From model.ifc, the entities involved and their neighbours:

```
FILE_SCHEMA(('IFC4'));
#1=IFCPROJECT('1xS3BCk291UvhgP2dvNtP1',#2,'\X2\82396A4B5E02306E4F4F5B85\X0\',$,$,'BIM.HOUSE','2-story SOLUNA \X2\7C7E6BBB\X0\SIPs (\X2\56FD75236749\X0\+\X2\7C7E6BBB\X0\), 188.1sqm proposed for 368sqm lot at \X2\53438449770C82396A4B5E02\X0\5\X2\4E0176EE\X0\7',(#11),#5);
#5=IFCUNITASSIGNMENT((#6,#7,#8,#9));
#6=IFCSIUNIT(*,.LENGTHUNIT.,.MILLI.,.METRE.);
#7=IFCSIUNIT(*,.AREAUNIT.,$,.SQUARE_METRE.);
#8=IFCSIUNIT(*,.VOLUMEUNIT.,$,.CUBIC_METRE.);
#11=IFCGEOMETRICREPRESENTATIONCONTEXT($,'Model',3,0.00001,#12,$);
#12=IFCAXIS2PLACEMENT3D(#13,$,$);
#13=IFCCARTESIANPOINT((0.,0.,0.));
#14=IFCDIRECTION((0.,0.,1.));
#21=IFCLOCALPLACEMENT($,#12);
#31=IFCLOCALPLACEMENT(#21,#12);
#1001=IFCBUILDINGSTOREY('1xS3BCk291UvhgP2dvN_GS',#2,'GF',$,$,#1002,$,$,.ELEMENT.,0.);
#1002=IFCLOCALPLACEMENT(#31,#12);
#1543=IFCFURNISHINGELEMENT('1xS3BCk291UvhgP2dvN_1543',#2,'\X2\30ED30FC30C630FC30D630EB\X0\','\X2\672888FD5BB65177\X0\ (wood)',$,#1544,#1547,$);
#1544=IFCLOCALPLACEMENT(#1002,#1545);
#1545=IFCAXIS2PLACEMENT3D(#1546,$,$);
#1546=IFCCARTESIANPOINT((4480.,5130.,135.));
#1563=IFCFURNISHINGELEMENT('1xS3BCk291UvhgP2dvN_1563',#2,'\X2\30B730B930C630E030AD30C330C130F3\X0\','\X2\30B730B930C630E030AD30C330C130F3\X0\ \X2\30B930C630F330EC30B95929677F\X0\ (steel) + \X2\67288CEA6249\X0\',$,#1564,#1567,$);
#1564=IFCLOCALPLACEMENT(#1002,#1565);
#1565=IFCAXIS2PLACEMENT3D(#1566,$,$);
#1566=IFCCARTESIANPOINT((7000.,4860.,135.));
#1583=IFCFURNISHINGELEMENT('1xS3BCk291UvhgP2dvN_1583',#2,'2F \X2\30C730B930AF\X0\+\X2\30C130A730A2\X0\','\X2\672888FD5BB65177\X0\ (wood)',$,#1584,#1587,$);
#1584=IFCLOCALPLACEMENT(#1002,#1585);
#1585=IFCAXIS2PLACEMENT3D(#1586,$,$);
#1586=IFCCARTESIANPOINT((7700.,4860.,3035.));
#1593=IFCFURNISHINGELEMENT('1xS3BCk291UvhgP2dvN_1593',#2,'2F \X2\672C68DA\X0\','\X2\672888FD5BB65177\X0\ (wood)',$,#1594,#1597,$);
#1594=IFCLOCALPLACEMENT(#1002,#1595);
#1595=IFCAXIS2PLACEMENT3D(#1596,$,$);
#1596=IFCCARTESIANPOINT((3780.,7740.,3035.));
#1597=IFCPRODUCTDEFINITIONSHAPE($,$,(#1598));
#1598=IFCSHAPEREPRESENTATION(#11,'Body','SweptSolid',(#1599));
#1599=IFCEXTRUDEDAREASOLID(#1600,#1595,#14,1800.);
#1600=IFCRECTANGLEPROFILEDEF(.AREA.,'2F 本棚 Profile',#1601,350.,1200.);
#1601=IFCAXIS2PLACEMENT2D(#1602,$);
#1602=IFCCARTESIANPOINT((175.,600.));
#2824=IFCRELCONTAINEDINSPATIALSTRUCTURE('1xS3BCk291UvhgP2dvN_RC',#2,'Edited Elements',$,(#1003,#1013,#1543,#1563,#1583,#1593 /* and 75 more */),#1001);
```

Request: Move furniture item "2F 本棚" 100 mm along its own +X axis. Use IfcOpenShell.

```python
import ifcopenshell
import ifcopenshell.api.geometry
import ifcopenshell.util.placement
import ifcopenshell.util.unit

model = ifcopenshell.open("model.ifc")
unit_scale = ifcopenshell.util.unit.calculate_unit_scale(model)

item = model.by_guid("1xS3BCk291UvhgP2dvN_1593")
matrix = ifcopenshell.util.placement.get_local_placement(item.ObjectPlacement)
matrix[:3, 3] += matrix[:3, 0] * 0.1 / unit_scale
ifcopenshell.api.geometry.edit_object_placement(model, product=item, matrix=matrix, is_si=False)

print(ifcopenshell.util.placement.get_local_placement(item.ObjectPlacement).round(3) + 0.0)

model.write("model_edited.ifc")
```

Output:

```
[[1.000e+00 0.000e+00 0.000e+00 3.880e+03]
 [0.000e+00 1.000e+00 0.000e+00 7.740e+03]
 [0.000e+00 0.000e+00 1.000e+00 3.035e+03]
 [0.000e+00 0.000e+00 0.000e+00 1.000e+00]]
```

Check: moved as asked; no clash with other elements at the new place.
